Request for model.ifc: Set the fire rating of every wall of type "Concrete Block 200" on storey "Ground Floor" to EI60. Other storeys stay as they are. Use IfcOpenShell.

First a look at what the model holds.

```python
import ifcopenshell
import ifcopenshell.util.element

model = ifcopenshell.open("model.ifc")
print(model.schema)
storey = next(s for s in model.by_type("IfcBuildingStorey") if s.Name == "Ground Floor")
walls = [e for e in ifcopenshell.util.element.get_decomposition(storey) if e.is_a("IfcWall")]
seen = {}
for e in walls:
    element_type = ifcopenshell.util.element.get_type(e)
    key = (element_type.Name if element_type != e and element_type else None, ifcopenshell.util.element.get_pset(e, "Pset_WallCommon", "FireRating"))
    seen[key] = seen.get(key, 0) + 1
for (name, value), count in sorted(seen.items(), key=str):
    print(count, "x", name, "|", value)
```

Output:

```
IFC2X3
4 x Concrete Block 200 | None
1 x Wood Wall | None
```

```python
import ifcopenshell
import ifcopenshell.api.pset
import ifcopenshell.util.element

model = ifcopenshell.open("model.ifc")

storey = next(s for s in model.by_type("IfcBuildingStorey") if s.Name == "Ground Floor")
walls = [e for e in ifcopenshell.util.element.get_decomposition(storey) if e.is_a("IfcWall")]

count = 0
for e in walls:
    element_type = ifcopenshell.util.element.get_type(e)
    if element_type in (None, e) or element_type.Name != "Concrete Block 200":
        continue
    # add_pset returns the element's existing set when there is one.
    pset = ifcopenshell.api.pset.add_pset(model, product=e, name="Pset_WallCommon")
    ifcopenshell.api.pset.edit_pset(model, pset=pset, properties={"FireRating": "EI60"})
    count += 1

print(count, "walls updated")

model.write("model_v2.ifc")
```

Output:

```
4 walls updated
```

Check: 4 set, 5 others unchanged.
